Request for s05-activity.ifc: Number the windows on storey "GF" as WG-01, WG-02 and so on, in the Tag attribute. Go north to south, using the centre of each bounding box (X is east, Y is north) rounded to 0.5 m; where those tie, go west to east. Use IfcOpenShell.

First a look at what the model holds.

```python
import ifcopenshell
import ifcopenshell.util.element
import ifcopenshell.util.placement

model = ifcopenshell.open("s05-activity.ifc")
print(model.schema)
storey = next(s for s in model.by_type("IfcBuildingStorey") if s.Name == "GF")
windows = [e for e in ifcopenshell.util.element.get_decomposition(storey) if e.is_a("IfcWindow")]
for e in sorted(windows, key=lambda e: e.id()):
    origin = ifcopenshell.util.placement.get_local_placement(e.ObjectPlacement)[:3, 3]
    print(e.id(), e.Tag, e.Name, origin.round(2) + 0.0, sep=" | ")
```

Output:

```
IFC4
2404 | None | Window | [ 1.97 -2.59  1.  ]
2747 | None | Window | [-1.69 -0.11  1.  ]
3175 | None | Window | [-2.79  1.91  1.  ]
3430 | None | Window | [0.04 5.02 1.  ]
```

```python
import ifcopenshell
import ifcopenshell.geom
import ifcopenshell.util.element
import ifcopenshell.util.shape

model = ifcopenshell.open("s05-activity.ifc")
settings = ifcopenshell.geom.settings()
settings.set("use-world-coords", True)


def centre(element):
    shape = ifcopenshell.geom.create_shape(settings, element)
    return ifcopenshell.util.shape.get_bbox_centroid(shape.geometry)


storey = next(s for s in model.by_type("IfcBuildingStorey") if s.Name == "GF")
windows = [e for e in ifcopenshell.util.element.get_decomposition(storey) if e.is_a("IfcWindow")]

# Insertion points can sit at a corner or the storey origin, so sort by the geometry (in metres).
centres = {e: centre(e) for e in windows}
windows.sort(key=lambda e: (-round(centres[e][1] / 0.5), centres[e][0]))

for i, e in enumerate(windows, start=1):
    number = f"WG-{i:02d}"
    e.Tag = number
    print(e.id(), number)

model.write("s05-activity_updated.ifc")
```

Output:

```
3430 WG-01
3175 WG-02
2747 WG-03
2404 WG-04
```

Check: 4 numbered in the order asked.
